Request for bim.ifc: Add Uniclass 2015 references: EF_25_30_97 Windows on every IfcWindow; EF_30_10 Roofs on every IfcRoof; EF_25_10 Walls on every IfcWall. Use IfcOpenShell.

First a look at what the model holds.

```python
import ifcopenshell

model = ifcopenshell.open("bim.ifc")
print(model.schema)
print("classifications:", [c.Name for c in model.by_type("IfcClassification")])
for ifc_class in ("IfcDoor", "IfcRoof", "IfcStair", "IfcWall", "IfcWindow"):
    print(ifc_class, len(model.by_type(ifc_class)))
```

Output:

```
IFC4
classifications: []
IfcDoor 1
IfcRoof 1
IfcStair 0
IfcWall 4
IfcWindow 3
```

```python
import ifcopenshell
import ifcopenshell.api.classification

model = ifcopenshell.open("bim.ifc")

system = ifcopenshell.api.classification.add_classification(model, classification="Uniclass 2015")

codes = {
    "IfcWindow": ("EF_25_30_97", "Windows"),
    "IfcRoof": ("EF_30_10", "Roofs"),
    "IfcWall": ("EF_25_10", "Walls"),
}
for ifc_class, (code, name) in codes.items():
    products = model.by_type(ifc_class)
    ifcopenshell.api.classification.add_reference(
        model, products=products, classification=system, identification=code, name=name
    )
    print(code, len(products))

model.write("bim-out.ifc")
```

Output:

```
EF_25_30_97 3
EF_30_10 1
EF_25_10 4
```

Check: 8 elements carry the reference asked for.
